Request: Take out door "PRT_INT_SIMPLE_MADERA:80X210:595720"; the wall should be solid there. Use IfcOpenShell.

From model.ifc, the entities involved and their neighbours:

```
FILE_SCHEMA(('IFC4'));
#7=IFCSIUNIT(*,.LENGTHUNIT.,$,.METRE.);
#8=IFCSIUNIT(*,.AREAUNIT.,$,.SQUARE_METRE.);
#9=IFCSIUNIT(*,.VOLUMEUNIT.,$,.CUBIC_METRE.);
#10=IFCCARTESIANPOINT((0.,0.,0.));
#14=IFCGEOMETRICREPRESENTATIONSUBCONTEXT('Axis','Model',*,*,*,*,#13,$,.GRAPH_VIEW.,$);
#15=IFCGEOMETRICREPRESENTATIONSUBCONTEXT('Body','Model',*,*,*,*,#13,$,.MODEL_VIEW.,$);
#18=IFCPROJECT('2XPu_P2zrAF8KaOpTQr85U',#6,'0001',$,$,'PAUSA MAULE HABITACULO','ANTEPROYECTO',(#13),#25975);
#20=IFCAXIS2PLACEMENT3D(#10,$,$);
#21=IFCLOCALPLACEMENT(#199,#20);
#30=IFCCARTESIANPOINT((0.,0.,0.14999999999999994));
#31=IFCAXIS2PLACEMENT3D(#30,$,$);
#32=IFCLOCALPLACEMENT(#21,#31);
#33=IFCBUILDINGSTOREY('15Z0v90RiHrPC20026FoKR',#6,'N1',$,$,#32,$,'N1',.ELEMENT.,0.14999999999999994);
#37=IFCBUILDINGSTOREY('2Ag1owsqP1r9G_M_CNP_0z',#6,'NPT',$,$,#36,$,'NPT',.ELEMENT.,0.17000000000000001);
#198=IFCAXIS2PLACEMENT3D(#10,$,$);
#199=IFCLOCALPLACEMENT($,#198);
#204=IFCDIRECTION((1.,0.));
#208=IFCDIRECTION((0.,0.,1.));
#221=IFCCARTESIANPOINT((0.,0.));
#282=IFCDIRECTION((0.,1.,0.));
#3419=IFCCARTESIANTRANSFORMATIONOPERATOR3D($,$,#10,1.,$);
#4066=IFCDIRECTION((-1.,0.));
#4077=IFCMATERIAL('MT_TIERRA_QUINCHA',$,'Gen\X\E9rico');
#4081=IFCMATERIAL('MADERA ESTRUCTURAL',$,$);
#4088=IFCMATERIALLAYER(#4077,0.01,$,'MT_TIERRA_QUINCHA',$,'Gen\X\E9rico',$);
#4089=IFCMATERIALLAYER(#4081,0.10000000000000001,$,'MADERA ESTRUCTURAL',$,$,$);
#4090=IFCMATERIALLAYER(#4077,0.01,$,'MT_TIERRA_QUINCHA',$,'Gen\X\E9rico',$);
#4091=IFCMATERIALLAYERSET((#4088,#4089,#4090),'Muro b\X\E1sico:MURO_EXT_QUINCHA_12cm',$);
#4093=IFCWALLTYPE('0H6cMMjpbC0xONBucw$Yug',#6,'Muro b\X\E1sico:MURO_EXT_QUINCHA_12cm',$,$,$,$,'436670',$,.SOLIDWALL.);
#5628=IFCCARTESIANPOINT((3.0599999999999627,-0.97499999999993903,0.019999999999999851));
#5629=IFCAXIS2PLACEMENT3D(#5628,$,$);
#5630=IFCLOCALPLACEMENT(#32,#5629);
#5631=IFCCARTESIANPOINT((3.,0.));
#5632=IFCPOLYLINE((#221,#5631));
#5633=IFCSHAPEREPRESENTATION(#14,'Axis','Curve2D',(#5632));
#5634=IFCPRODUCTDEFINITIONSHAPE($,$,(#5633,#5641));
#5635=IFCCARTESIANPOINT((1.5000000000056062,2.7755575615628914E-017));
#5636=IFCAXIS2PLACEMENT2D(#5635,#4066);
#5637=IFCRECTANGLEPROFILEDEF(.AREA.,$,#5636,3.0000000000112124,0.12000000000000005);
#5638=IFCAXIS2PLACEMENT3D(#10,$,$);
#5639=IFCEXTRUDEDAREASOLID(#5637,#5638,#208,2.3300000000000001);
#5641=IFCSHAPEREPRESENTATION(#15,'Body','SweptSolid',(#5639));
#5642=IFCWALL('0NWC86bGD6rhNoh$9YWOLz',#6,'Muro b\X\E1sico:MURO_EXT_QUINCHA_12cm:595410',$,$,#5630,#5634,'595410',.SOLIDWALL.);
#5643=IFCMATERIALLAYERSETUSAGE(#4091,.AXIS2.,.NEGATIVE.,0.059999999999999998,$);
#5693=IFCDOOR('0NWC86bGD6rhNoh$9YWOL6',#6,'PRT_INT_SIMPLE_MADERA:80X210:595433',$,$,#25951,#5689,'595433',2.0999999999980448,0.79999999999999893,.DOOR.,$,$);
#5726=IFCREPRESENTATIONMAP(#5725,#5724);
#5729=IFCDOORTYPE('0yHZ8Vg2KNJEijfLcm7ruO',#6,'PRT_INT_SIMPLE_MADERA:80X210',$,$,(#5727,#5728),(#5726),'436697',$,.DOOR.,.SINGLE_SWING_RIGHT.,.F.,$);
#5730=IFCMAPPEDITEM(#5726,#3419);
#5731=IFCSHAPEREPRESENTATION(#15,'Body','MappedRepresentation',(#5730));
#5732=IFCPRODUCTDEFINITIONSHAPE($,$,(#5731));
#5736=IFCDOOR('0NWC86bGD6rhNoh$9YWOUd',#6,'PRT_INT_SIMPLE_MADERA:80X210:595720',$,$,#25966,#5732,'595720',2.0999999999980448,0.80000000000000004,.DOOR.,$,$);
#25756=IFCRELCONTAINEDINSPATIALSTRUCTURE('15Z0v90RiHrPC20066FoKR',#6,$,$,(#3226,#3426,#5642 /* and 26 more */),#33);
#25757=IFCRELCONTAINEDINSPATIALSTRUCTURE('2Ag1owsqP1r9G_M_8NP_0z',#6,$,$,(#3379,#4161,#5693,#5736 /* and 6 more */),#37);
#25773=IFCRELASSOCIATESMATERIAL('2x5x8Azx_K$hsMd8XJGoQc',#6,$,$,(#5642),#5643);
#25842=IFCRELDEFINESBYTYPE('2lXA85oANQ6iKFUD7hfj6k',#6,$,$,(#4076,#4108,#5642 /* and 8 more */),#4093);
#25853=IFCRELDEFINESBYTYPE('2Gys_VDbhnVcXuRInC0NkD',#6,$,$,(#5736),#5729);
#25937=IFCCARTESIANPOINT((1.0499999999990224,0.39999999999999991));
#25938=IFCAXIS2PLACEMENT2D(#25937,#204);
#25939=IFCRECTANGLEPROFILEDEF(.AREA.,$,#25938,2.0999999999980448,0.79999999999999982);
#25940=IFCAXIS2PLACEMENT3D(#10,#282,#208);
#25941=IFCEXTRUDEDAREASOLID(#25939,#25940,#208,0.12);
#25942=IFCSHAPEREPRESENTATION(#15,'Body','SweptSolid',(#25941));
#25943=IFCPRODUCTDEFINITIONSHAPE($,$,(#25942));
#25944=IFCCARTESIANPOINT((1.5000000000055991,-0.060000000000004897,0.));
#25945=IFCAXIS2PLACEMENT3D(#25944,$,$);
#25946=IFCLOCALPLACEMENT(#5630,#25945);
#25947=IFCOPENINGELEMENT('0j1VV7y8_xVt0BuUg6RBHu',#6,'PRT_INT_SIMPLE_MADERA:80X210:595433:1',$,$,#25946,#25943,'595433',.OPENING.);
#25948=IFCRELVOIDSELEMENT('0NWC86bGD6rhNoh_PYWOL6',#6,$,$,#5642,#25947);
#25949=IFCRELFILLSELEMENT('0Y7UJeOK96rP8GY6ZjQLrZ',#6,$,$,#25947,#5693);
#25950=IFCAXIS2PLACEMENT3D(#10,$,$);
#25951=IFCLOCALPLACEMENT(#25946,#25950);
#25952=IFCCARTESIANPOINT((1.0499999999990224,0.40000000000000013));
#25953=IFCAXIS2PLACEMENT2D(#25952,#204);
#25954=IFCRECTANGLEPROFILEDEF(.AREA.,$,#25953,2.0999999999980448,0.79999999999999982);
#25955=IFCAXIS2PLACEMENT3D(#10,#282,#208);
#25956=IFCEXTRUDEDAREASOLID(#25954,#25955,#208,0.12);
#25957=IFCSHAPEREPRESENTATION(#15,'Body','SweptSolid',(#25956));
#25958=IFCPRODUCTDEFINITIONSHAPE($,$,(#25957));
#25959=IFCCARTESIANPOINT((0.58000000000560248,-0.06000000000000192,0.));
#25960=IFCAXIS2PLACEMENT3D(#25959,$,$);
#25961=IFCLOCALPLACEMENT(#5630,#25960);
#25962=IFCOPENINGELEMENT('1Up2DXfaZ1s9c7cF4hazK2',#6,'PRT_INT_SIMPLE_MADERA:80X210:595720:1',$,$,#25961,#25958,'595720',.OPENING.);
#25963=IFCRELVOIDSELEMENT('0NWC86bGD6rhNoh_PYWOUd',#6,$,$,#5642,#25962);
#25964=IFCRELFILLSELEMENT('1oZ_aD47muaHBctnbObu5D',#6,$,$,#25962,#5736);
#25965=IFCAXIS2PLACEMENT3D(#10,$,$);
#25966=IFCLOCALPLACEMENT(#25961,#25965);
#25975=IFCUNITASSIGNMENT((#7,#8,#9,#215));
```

```python
import ifcopenshell
import ifcopenshell.api.feature
import ifcopenshell.api.root
import ifcopenshell.geom
import ifcopenshell.util.shape

model = ifcopenshell.open("model.ifc")
settings = ifcopenshell.geom.settings()


def volume(element):
    """Net volume in cubic metres, openings subtracted."""
    shape = ifcopenshell.geom.create_shape(settings, element)
    return ifcopenshell.util.shape.get_volume(shape.geometry)


door = model.by_guid("0NWC86bGD6rhNoh$9YWOUd")
opening = door.FillsVoids[0].RelatingOpeningElement
wall = opening.VoidsElements[0].RelatingBuildingElement
before = volume(wall)

ifcopenshell.api.root.remove_product(model, product=door)
ifcopenshell.api.feature.remove_feature(model, feature=opening)

after = volume(wall)

print(f"wall volume {before:.3f} -> {after:.3f} m3")

model.write("model_rev.ifc")
```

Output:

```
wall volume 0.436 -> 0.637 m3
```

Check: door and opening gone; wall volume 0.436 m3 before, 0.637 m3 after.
